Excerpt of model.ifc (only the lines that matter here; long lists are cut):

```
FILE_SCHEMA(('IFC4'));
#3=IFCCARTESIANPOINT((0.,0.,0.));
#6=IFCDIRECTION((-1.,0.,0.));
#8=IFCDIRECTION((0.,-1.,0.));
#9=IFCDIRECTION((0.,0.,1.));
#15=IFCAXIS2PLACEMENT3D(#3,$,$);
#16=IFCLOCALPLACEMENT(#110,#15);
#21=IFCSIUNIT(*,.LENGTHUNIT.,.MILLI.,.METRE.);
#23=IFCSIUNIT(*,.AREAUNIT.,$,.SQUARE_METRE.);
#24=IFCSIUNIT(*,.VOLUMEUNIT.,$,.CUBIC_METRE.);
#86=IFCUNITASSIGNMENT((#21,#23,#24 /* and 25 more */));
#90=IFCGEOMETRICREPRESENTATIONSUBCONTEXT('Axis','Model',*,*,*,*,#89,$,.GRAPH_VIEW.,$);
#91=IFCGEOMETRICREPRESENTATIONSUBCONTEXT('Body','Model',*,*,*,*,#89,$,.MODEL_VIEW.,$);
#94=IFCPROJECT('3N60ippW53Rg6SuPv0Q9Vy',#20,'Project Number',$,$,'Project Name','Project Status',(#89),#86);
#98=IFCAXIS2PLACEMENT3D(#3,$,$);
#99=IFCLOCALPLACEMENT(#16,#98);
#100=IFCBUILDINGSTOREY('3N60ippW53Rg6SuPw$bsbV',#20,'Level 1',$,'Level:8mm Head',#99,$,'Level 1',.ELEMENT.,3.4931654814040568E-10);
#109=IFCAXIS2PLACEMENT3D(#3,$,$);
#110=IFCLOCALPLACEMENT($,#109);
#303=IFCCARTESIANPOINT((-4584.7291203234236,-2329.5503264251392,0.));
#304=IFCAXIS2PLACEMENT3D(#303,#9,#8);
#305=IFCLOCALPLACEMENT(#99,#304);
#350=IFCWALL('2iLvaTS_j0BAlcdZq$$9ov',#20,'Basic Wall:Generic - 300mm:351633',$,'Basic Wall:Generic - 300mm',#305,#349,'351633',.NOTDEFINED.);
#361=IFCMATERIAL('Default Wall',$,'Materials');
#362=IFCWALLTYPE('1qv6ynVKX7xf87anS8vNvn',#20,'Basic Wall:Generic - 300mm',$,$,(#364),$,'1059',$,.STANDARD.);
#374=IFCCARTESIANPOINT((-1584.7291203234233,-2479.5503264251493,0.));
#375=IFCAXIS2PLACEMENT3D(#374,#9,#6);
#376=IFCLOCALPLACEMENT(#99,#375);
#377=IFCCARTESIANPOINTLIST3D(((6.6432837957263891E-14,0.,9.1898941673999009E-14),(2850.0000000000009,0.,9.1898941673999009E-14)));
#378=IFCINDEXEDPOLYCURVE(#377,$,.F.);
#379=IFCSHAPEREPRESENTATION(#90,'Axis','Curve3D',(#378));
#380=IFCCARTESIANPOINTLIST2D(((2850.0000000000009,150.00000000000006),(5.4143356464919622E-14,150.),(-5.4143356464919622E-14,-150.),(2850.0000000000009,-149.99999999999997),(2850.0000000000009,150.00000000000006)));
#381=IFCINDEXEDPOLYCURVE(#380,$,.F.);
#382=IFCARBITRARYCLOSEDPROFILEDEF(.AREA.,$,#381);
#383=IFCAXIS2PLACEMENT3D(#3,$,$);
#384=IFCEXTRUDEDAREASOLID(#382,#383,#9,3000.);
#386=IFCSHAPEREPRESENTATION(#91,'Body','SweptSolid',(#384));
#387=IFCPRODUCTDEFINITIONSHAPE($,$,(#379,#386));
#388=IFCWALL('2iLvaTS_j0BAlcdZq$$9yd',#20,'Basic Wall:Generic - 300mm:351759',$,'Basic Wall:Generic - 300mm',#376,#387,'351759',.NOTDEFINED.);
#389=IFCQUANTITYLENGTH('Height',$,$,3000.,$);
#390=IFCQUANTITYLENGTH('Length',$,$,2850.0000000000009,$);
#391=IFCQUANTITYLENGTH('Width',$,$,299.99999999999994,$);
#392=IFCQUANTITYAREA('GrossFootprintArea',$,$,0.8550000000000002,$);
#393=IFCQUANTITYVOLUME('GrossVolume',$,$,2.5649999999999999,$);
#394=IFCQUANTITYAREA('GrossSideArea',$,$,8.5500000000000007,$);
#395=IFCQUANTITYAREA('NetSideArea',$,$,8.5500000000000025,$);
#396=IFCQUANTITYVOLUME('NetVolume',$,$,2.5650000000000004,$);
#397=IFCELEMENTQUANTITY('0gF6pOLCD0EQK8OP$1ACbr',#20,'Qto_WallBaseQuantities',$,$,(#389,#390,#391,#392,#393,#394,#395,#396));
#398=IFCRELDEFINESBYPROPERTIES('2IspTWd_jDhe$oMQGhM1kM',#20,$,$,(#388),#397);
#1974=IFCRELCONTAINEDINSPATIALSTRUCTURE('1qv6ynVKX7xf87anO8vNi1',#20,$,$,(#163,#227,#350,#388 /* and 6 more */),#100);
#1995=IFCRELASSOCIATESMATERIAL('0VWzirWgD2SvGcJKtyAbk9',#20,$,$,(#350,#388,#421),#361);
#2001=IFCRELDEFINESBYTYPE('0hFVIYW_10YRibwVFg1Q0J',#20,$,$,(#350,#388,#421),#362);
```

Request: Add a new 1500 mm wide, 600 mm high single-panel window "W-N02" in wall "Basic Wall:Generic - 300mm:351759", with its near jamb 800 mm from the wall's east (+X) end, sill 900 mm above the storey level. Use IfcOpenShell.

```python
import numpy as np
import ifcopenshell
import ifcopenshell.api.feature
import ifcopenshell.api.geometry
import ifcopenshell.api.pset
import ifcopenshell.api.root
import ifcopenshell.api.spatial
import ifcopenshell.geom
import ifcopenshell.util.element
import ifcopenshell.util.placement
import ifcopenshell.util.representation
import ifcopenshell.util.shape
import ifcopenshell.util.unit

model = ifcopenshell.open("model.ifc")
unit_scale = ifcopenshell.util.unit.calculate_unit_scale(model)
area_scale = ifcopenshell.util.unit.calculate_unit_scale(model, "AREAUNIT")
volume_scale = ifcopenshell.util.unit.calculate_unit_scale(model, "VOLUMEUNIT")
settings = ifcopenshell.geom.settings()


def volume(element):
    """Net volume in cubic metres, openings subtracted."""
    shape = ifcopenshell.geom.create_shape(settings, element)
    return ifcopenshell.util.shape.get_volume(shape.geometry)


wall = model.by_guid("2iLvaTS_j0BAlcdZq$$9yd")
storey = ifcopenshell.util.element.get_container(wall, ifc_class="IfcBuildingStorey")
context = ifcopenshell.util.representation.get_context(model, "Model", "Body", "MODEL_VIEW")
before = volume(wall)

width, height, from_end, sill = 1.5, 0.6, 0.8, 0.9  # metres

# The wall runs along its own X axis, and the end named is its -X end.
wall_shape = ifcopenshell.geom.create_shape(settings, wall)
x, y, z = ifcopenshell.util.shape.get_vertices(wall_shape.geometry).T
start = x.min() + from_end
face, thickness = float(y.min()), float(y.max() - y.min())
wall_matrix = ifcopenshell.util.placement.get_local_placement(wall.ObjectPlacement)
level = ifcopenshell.util.placement.get_local_placement(storey.ObjectPlacement)[2, 3]


def in_wall(x, y):
    """Placement at x, y metres in the wall's axes, at sill height."""
    matrix = wall_matrix.copy()
    matrix[:, 3] = wall_matrix @ np.array([x / unit_scale, y / unit_scale, 0.0, 1.0])
    matrix[2, 3] = level + sill / unit_scale
    return matrix


# Opening: a box that overshoots both wall faces by 50 mm.
opening = ifcopenshell.api.root.create_entity(model, ifc_class="IfcOpeningElement", predefined_type="OPENING")
box = ifcopenshell.api.geometry.add_wall_representation(
    model, context=context, length=width, height=height, thickness=thickness + 0.1
)
ifcopenshell.api.geometry.assign_representation(model, product=opening, representation=box)
ifcopenshell.api.geometry.edit_object_placement(model, product=opening, matrix=in_wall(start, face - 0.05), is_si=False)
ifcopenshell.api.feature.add_feature(model, feature=opening, element=wall)

window = ifcopenshell.api.root.create_entity(model, ifc_class="IfcWindow", name="W-N02", predefined_type="WINDOW")
window.OverallWidth, window.OverallHeight = width / unit_scale, height / unit_scale
window.PartitioningType = "SINGLE_PANEL"
body = ifcopenshell.api.geometry.add_window_representation(
    model,
    context=context,
    overall_width=window.OverallWidth,
    overall_height=window.OverallHeight,
    partition_type="SINGLE_PANEL",
)
ifcopenshell.api.geometry.assign_representation(model, product=window, representation=body)
ifcopenshell.api.spatial.assign_container(model, products=[window], relating_structure=storey)
ifcopenshell.api.feature.add_filling(model, opening=opening, element=window)

# Centre the window in the wall's thickness.
ifcopenshell.api.geometry.edit_object_placement(model, product=window, matrix=in_wall(start, face), is_si=False)
window_shape = ifcopenshell.geom.create_shape(settings, window)
depth = ifcopenshell.util.shape.get_vertices(window_shape.geometry)[:, 1]
offset = face + thickness / 2 - (depth.min() + depth.max()) / 2
ifcopenshell.api.geometry.edit_object_placement(model, product=window, matrix=in_wall(start, offset), is_si=False)

after = volume(wall)

# Update the wall's stored quantities.
qto = model.by_id(ifcopenshell.util.element.get_pset(wall, "Qto_WallBaseQuantities", should_inherit=False)["id"])
ifcopenshell.api.pset.edit_qto(model, qto=qto, properties={
    "NetSideArea": after / thickness / area_scale,
    "NetVolume": after / volume_scale,
})

print(f"wall volume {before:.3f} -> {after:.3f} m3")

model.write("model_v2.ifc")
```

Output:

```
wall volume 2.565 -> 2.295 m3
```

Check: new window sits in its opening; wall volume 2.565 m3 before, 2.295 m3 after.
